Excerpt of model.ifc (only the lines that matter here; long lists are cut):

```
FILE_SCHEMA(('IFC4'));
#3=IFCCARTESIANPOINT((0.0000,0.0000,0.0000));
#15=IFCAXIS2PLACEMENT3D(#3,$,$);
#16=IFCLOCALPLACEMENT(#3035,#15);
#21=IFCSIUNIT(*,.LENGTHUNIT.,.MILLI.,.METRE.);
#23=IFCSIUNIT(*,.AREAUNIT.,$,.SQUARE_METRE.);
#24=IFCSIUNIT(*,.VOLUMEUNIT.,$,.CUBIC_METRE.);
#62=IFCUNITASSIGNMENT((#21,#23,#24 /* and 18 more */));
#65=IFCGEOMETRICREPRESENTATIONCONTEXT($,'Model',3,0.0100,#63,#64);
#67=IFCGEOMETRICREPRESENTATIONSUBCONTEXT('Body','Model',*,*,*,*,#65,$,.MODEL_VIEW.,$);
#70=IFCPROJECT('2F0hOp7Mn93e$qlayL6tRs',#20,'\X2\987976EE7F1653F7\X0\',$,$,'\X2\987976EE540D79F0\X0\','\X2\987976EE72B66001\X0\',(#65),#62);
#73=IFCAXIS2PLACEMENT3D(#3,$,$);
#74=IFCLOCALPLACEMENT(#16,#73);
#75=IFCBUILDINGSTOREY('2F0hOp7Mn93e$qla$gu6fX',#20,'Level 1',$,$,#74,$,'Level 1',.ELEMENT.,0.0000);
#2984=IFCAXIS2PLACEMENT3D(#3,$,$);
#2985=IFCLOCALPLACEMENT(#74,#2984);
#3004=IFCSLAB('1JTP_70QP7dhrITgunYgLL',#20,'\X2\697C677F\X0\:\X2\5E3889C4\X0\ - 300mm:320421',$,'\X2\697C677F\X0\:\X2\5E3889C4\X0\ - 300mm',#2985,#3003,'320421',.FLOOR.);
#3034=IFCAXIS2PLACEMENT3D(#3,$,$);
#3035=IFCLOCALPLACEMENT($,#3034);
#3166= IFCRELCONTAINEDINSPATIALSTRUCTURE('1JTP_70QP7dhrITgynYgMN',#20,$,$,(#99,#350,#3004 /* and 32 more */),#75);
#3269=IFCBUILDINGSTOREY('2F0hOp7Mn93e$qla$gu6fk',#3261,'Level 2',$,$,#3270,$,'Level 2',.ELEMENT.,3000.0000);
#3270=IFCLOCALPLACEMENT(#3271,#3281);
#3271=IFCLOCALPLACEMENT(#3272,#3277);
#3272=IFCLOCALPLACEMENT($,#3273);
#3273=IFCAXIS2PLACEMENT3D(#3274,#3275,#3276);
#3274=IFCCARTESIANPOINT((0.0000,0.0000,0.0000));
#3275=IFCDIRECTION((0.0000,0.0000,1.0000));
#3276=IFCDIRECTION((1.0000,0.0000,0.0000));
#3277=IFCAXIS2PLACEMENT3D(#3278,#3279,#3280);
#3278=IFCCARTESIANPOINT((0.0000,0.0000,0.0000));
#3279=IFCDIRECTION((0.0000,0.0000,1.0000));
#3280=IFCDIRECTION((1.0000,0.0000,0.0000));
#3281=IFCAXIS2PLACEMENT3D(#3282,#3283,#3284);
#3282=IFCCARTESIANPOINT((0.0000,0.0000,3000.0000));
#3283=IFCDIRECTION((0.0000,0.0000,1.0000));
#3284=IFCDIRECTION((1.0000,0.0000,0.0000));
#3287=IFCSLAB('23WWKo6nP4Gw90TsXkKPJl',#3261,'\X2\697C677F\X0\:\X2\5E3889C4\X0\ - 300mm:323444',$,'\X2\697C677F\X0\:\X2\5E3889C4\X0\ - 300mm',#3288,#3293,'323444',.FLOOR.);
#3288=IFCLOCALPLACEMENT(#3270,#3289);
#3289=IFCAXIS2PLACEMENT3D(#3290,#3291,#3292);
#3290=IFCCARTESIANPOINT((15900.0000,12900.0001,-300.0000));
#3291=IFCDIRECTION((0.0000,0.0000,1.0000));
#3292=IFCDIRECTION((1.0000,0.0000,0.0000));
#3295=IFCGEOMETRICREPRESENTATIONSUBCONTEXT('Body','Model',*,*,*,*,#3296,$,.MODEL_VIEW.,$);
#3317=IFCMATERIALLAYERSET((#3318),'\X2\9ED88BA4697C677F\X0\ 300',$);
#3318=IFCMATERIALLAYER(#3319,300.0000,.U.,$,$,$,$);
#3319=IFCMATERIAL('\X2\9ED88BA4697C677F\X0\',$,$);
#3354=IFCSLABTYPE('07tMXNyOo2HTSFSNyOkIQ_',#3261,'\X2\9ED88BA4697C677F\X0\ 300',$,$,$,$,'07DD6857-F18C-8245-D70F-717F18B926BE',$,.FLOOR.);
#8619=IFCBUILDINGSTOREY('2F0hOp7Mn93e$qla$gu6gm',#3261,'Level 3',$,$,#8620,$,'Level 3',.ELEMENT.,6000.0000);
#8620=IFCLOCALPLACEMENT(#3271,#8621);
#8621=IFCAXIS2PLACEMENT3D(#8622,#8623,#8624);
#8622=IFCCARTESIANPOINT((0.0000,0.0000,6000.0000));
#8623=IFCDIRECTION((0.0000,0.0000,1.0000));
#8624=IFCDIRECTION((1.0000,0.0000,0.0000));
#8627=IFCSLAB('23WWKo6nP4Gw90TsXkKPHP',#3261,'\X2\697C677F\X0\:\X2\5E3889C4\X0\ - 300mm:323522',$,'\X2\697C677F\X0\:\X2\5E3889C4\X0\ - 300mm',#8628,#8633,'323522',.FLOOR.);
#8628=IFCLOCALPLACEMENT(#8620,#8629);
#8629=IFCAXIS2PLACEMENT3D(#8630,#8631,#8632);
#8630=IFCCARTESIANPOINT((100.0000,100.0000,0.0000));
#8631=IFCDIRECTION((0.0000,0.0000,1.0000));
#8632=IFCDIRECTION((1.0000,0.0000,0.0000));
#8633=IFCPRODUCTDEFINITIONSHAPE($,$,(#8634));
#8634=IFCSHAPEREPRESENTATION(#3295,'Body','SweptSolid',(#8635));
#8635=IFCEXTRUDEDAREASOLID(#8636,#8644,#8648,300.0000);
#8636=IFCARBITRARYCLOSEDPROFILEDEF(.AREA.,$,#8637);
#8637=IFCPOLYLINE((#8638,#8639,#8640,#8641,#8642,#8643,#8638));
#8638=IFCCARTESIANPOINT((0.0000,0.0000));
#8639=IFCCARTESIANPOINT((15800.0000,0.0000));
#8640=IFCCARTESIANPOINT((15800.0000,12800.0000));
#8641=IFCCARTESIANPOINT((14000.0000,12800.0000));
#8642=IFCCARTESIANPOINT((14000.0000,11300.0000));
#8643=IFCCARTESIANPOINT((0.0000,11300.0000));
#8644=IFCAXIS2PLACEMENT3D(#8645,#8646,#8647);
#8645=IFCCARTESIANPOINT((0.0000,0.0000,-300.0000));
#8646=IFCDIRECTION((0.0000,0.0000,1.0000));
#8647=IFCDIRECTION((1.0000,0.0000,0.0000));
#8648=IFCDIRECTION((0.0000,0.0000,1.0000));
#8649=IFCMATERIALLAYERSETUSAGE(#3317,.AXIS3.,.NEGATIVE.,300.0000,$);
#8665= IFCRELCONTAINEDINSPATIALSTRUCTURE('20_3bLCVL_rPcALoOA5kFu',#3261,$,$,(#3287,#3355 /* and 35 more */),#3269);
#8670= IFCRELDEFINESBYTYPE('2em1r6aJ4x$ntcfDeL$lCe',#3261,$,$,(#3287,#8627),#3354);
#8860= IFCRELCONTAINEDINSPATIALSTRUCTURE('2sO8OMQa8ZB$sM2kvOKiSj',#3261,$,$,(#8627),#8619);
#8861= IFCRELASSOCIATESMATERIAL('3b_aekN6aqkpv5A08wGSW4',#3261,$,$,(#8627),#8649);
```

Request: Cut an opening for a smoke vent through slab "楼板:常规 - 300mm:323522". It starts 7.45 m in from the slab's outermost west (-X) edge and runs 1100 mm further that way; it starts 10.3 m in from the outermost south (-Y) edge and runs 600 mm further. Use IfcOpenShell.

```python
import numpy as np
import ifcopenshell
import ifcopenshell.api.feature
import ifcopenshell.api.geometry
import ifcopenshell.api.root
import ifcopenshell.geom
import ifcopenshell.util.placement
import ifcopenshell.util.representation
import ifcopenshell.util.shape
import ifcopenshell.util.unit

model = ifcopenshell.open("model.ifc")
unit_scale = ifcopenshell.util.unit.calculate_unit_scale(model)
settings = ifcopenshell.geom.settings()


def volume(element):
    """Net volume in cubic metres, openings subtracted."""
    shape = ifcopenshell.geom.create_shape(settings, element)
    return ifcopenshell.util.shape.get_volume(shape.geometry)


slab = model.by_guid("23WWKo6nP4Gw90TsXkKPHP")
before = volume(slab)

# Extent in the slab's own axes, in metres. The edges named are its -X and -Y sides.
slab_shape = ifcopenshell.geom.create_shape(settings, slab)
vertices = ifcopenshell.util.shape.get_vertices(slab_shape.geometry)
x_min, y_min, bottom = vertices.min(axis=0)
top = vertices[:, 2].max()

opening = ifcopenshell.api.root.create_entity(model, ifc_class="IfcOpeningElement", name="Smoke vent opening", predefined_type="OPENING")
context = ifcopenshell.util.representation.get_context(model, "Model", "Body", "MODEL_VIEW")
width, depth = 1.1, 0.6
outline = [(0.0, 0.0), (width, 0.0), (width, depth), (0.0, depth), (0.0, 0.0)]
# Overshoot both faces by 50 mm so the cut is clean.
shape = ifcopenshell.api.geometry.add_slab_representation(
    model, context=context, depth=top - bottom + 0.1, polyline=outline
)
ifcopenshell.api.geometry.assign_representation(model, product=opening, representation=shape)

matrix = ifcopenshell.util.placement.get_local_placement(slab.ObjectPlacement)
matrix[:, 3] = matrix @ np.append(np.array([x_min + 7.45, y_min + 10.3, bottom - 0.05]) / unit_scale, 1.0)
ifcopenshell.api.geometry.edit_object_placement(model, product=opening, matrix=matrix, is_si=False)
ifcopenshell.api.feature.add_feature(model, feature=opening, element=slab)

after = volume(slab)

print(f"slab volume {before:.3f} -> {after:.3f} m3")

model.write("model_v2.ifc")
```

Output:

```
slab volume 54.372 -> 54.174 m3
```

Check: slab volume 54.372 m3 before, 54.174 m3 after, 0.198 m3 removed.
